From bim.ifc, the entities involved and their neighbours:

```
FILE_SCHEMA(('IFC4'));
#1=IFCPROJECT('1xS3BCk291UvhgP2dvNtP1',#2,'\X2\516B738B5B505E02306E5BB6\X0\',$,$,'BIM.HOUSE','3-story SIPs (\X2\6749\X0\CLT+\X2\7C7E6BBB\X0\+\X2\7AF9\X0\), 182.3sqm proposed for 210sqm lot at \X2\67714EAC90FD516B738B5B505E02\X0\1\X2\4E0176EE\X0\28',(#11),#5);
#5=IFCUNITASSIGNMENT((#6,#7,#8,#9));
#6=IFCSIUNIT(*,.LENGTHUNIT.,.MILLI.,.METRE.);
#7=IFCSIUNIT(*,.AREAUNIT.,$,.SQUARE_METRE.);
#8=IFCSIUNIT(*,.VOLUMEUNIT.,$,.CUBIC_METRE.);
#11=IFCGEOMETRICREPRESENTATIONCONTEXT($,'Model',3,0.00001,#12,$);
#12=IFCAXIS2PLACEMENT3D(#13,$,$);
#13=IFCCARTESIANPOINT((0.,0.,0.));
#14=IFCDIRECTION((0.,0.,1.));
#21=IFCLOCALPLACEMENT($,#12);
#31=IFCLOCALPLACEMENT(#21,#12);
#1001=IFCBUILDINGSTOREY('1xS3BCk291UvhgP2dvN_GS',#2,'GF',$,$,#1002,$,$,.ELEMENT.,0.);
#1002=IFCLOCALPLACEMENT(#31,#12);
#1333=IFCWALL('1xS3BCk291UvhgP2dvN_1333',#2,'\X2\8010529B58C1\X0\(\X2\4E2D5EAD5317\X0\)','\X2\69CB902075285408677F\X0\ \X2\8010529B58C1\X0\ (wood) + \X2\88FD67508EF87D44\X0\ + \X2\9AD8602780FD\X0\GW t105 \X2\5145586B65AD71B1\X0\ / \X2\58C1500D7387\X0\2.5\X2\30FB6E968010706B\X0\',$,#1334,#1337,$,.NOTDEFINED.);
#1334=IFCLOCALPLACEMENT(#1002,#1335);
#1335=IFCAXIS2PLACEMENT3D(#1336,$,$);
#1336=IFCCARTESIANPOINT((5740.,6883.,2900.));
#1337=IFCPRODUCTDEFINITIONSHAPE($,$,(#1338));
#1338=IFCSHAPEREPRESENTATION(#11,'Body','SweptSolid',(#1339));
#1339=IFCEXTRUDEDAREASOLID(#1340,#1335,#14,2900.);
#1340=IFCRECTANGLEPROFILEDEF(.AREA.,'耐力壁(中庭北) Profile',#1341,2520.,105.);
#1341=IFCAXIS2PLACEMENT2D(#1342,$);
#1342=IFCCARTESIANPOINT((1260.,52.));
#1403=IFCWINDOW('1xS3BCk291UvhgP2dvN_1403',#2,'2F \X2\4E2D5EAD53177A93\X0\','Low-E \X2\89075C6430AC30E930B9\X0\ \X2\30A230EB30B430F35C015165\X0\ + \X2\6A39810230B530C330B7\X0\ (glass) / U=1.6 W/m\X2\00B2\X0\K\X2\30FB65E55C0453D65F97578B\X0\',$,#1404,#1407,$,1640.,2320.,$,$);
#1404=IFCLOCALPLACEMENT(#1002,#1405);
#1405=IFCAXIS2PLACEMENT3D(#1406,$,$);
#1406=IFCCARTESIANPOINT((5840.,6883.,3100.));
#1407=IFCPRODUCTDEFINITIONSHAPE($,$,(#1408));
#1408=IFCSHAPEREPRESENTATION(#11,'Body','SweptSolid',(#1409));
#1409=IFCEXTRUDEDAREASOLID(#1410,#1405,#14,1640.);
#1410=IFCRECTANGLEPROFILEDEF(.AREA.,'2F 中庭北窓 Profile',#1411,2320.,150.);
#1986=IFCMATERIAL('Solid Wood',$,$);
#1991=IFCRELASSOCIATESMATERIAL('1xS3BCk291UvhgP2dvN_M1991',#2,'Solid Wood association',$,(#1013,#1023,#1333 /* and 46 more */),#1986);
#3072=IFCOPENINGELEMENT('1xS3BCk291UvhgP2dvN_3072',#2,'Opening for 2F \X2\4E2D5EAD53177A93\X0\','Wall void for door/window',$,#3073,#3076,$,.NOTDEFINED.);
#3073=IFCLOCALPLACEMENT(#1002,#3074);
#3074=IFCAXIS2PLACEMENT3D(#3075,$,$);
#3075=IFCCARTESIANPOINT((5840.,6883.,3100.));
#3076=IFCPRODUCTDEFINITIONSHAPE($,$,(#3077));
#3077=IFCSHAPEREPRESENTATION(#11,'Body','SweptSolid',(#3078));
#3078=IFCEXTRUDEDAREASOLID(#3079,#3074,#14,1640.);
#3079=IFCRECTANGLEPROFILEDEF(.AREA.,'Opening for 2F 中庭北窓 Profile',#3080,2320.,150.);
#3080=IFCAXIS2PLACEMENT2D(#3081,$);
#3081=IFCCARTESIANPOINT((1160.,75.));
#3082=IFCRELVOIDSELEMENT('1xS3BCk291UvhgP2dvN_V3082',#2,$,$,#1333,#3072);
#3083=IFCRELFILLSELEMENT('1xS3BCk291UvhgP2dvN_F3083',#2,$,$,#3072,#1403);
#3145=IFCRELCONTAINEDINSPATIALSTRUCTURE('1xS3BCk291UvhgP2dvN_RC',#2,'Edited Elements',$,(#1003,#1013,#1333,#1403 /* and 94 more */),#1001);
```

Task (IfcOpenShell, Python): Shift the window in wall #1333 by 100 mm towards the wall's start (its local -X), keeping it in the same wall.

```python
import ifcopenshell
import ifcopenshell.api.geometry
import ifcopenshell.util.placement
import ifcopenshell.util.unit

model = ifcopenshell.open("bim.ifc")
unit_scale = ifcopenshell.util.unit.calculate_unit_scale(model)

window = model.by_guid("1xS3BCk291UvhgP2dvN_1403")
opening = window.FillsVoids[0].RelatingOpeningElement
wall = opening.VoidsElements[0].RelatingBuildingElement

wall_matrix = ifcopenshell.util.placement.get_local_placement(wall.ObjectPlacement)
shift = wall_matrix[:3, 0] * -0.1 / unit_scale
before = ifcopenshell.util.placement.get_local_placement(window.ObjectPlacement)[:3, 3].copy()

# The window is not placed relative to its opening, so move both.
for product in (opening, window):
    matrix = ifcopenshell.util.placement.get_local_placement(product.ObjectPlacement)
    matrix[:3, 3] += shift
    ifcopenshell.api.geometry.edit_object_placement(model, product=product, matrix=matrix, is_si=False)

after = ifcopenshell.util.placement.get_local_placement(window.ObjectPlacement)[:3, 3]
print("window moved by", (after - before).round(3) + 0.0)

model.write("bim_edited.ifc")
```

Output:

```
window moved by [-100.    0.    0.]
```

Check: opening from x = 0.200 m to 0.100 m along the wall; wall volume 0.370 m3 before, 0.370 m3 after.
